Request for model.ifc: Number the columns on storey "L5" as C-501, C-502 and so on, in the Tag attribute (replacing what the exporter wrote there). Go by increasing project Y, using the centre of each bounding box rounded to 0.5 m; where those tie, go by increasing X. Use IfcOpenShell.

First a look at what the model holds.

```python
import ifcopenshell
import ifcopenshell.util.element
import ifcopenshell.util.placement

model = ifcopenshell.open("model.ifc")
print(model.schema)
storey = next(s for s in model.by_type("IfcBuildingStorey") if s.Name == "L5")
columns = [e for e in ifcopenshell.util.element.get_decomposition(storey) if e.is_a("IfcColumn")]
for e in sorted(columns, key=lambda e: e.id()):
    origin = ifcopenshell.util.placement.get_local_placement(e.ObjectPlacement)[:3, 3]
    print(e.id(), e.Tag, e.Name, origin.round(2) + 0.0, sep=" | ")
```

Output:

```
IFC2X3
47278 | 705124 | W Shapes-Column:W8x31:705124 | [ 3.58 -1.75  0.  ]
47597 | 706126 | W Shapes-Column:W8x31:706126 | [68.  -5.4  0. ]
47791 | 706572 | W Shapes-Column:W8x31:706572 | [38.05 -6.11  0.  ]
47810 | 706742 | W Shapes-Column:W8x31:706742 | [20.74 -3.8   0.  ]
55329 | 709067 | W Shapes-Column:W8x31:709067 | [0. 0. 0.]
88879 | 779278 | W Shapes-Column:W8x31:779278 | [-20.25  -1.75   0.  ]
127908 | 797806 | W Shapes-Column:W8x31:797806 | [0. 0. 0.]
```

```python
import ifcopenshell
import ifcopenshell.geom
import ifcopenshell.util.element
import ifcopenshell.util.shape

model = ifcopenshell.open("model.ifc")
settings = ifcopenshell.geom.settings()
settings.set("use-world-coords", True)


def centre(element):
    shape = ifcopenshell.geom.create_shape(settings, element)
    return ifcopenshell.util.shape.get_bbox_centroid(shape.geometry)


storey = next(s for s in model.by_type("IfcBuildingStorey") if s.Name == "L5")
columns = [e for e in ifcopenshell.util.element.get_decomposition(storey) if e.is_a("IfcColumn")]

# Insertion points can sit at a corner or the storey origin, so sort by the geometry (in metres).
centres = {e: centre(e) for e in columns}
columns.sort(key=lambda e: (round(centres[e][1] / 0.5), centres[e][0]))

for i, e in enumerate(columns, start=1):
    number = f"C-5{i:02d}"
    e.Tag = number
    print(e.id(), number)

model.write("model_v2.ifc")
```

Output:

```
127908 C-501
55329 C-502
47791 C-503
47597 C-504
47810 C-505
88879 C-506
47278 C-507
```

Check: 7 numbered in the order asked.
